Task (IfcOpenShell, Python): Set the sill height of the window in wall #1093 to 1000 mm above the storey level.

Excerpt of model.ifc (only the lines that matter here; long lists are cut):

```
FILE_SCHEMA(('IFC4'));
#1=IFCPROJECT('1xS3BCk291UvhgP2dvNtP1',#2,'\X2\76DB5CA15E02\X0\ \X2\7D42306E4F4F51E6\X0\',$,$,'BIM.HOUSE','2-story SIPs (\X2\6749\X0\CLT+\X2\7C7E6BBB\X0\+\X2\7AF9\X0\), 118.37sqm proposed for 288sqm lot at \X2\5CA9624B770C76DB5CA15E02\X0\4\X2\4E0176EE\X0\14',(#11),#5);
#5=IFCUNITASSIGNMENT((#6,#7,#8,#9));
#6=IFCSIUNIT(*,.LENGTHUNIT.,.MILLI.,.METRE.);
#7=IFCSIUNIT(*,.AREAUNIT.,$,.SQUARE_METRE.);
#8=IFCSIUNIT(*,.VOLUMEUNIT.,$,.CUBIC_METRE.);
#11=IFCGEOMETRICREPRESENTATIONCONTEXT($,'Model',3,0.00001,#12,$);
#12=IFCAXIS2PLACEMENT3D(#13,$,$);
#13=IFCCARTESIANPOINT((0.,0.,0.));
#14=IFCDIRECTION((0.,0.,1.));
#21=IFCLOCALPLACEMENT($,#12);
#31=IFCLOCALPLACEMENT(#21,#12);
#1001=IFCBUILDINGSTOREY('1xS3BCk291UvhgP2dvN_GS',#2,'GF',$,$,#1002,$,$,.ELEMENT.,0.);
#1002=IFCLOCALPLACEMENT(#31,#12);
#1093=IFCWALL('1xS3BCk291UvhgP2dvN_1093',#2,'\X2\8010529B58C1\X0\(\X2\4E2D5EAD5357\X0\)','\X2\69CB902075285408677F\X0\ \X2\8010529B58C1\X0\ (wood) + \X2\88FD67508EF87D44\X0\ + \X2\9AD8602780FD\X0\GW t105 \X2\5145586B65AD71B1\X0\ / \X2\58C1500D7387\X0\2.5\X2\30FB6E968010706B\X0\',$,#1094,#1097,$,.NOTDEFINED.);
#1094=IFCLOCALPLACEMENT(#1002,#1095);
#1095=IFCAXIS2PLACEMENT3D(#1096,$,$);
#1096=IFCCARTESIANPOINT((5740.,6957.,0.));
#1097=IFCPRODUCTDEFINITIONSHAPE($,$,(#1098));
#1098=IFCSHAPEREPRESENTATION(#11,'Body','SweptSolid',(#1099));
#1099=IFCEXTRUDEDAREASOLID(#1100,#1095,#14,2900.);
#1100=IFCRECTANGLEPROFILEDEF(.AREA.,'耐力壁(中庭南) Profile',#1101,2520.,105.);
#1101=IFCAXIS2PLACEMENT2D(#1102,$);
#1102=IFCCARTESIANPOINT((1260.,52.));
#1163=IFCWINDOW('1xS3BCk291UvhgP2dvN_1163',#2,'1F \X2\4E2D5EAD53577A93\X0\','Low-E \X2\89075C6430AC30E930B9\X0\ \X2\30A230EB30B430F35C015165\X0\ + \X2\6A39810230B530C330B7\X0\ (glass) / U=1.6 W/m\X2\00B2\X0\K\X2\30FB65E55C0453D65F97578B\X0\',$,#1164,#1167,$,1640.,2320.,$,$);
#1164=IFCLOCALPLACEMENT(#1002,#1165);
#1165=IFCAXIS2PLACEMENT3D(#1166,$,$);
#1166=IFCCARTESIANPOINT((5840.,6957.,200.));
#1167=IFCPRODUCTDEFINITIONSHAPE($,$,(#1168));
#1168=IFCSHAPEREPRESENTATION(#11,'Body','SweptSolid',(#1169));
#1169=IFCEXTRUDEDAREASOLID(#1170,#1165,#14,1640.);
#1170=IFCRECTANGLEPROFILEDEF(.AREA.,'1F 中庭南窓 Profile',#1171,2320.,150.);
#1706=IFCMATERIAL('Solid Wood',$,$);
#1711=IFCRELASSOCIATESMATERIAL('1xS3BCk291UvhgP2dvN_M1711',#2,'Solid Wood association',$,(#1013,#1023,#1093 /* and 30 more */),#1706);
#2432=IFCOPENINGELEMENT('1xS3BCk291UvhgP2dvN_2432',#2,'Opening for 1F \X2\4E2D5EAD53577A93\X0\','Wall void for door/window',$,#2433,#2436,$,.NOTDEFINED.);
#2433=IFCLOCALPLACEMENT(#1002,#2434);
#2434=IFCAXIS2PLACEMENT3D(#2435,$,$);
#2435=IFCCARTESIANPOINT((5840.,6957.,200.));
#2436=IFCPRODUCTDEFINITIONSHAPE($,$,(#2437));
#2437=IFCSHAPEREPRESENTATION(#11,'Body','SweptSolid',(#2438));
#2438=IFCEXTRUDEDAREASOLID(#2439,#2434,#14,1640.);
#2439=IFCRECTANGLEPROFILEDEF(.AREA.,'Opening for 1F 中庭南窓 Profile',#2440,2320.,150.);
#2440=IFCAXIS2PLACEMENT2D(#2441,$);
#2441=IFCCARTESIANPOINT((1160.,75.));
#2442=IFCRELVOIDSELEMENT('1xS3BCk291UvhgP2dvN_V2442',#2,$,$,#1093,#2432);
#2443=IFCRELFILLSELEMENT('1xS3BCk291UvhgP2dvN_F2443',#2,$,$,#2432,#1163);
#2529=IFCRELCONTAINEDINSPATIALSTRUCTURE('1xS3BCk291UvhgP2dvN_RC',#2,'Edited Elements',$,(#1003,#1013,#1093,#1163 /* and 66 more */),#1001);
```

```python
import numpy as np
import ifcopenshell
import ifcopenshell.api.geometry
import ifcopenshell.geom
import ifcopenshell.util.element
import ifcopenshell.util.placement
import ifcopenshell.util.shape
import ifcopenshell.util.unit

model = ifcopenshell.open("model.ifc")
unit_scale = ifcopenshell.util.unit.calculate_unit_scale(model)

window = model.by_guid("1xS3BCk291UvhgP2dvN_1163")
opening = window.FillsVoids[0].RelatingOpeningElement
storey = ifcopenshell.util.element.get_container(window, ifc_class="IfcBuildingStorey")
level = ifcopenshell.util.placement.get_local_placement(storey.ObjectPlacement)[2, 3]

# The opening's origin need not be at the sill, so measure its lowest point.
shape = ifcopenshell.geom.create_shape(ifcopenshell.geom.settings(), opening)
bottom = ifcopenshell.util.shape.get_shape_bottom_elevation(shape, shape.geometry) / unit_scale
dz = level + 1 / unit_scale - bottom

shift = np.array([0.0, 0.0, dz])
# The window is not placed relative to its opening, so move both.
for product in (opening, window):
    matrix = ifcopenshell.util.placement.get_local_placement(product.ObjectPlacement)
    matrix[:3, 3] += shift
    ifcopenshell.api.geometry.edit_object_placement(model, product=product, matrix=matrix, is_si=False)

print(f"moved by {dz * unit_scale:+.3f} m")

model.write("model_v2.ifc")
```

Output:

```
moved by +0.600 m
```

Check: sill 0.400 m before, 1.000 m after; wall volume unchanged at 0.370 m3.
